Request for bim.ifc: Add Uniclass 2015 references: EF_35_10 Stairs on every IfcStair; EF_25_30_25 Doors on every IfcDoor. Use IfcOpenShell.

First a look at what the model holds.

```python
import ifcopenshell

model = ifcopenshell.open("bim.ifc")
print(model.schema)
print("classifications:", [c.Name for c in model.by_type("IfcClassification")])
for ifc_class in ("IfcDoor", "IfcRoof", "IfcStair", "IfcWall", "IfcWindow"):
    print(ifc_class, len(model.by_type(ifc_class)))
```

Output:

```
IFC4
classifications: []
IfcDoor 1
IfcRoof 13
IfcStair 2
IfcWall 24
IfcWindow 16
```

```python
import ifcopenshell
import ifcopenshell.api.classification

model = ifcopenshell.open("bim.ifc")

system = ifcopenshell.api.classification.add_classification(model, classification="Uniclass 2015")

codes = {
    "IfcStair": ("EF_35_10", "Stairs"),
    "IfcDoor": ("EF_25_30_25", "Doors"),
}
for ifc_class, (code, name) in codes.items():
    products = model.by_type(ifc_class)
    ifcopenshell.api.classification.add_reference(
        model, products=products, classification=system, identification=code, name=name
    )
    print(code, len(products))

model.write("bim_updated.ifc")
```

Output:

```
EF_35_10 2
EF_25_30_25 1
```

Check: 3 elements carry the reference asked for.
